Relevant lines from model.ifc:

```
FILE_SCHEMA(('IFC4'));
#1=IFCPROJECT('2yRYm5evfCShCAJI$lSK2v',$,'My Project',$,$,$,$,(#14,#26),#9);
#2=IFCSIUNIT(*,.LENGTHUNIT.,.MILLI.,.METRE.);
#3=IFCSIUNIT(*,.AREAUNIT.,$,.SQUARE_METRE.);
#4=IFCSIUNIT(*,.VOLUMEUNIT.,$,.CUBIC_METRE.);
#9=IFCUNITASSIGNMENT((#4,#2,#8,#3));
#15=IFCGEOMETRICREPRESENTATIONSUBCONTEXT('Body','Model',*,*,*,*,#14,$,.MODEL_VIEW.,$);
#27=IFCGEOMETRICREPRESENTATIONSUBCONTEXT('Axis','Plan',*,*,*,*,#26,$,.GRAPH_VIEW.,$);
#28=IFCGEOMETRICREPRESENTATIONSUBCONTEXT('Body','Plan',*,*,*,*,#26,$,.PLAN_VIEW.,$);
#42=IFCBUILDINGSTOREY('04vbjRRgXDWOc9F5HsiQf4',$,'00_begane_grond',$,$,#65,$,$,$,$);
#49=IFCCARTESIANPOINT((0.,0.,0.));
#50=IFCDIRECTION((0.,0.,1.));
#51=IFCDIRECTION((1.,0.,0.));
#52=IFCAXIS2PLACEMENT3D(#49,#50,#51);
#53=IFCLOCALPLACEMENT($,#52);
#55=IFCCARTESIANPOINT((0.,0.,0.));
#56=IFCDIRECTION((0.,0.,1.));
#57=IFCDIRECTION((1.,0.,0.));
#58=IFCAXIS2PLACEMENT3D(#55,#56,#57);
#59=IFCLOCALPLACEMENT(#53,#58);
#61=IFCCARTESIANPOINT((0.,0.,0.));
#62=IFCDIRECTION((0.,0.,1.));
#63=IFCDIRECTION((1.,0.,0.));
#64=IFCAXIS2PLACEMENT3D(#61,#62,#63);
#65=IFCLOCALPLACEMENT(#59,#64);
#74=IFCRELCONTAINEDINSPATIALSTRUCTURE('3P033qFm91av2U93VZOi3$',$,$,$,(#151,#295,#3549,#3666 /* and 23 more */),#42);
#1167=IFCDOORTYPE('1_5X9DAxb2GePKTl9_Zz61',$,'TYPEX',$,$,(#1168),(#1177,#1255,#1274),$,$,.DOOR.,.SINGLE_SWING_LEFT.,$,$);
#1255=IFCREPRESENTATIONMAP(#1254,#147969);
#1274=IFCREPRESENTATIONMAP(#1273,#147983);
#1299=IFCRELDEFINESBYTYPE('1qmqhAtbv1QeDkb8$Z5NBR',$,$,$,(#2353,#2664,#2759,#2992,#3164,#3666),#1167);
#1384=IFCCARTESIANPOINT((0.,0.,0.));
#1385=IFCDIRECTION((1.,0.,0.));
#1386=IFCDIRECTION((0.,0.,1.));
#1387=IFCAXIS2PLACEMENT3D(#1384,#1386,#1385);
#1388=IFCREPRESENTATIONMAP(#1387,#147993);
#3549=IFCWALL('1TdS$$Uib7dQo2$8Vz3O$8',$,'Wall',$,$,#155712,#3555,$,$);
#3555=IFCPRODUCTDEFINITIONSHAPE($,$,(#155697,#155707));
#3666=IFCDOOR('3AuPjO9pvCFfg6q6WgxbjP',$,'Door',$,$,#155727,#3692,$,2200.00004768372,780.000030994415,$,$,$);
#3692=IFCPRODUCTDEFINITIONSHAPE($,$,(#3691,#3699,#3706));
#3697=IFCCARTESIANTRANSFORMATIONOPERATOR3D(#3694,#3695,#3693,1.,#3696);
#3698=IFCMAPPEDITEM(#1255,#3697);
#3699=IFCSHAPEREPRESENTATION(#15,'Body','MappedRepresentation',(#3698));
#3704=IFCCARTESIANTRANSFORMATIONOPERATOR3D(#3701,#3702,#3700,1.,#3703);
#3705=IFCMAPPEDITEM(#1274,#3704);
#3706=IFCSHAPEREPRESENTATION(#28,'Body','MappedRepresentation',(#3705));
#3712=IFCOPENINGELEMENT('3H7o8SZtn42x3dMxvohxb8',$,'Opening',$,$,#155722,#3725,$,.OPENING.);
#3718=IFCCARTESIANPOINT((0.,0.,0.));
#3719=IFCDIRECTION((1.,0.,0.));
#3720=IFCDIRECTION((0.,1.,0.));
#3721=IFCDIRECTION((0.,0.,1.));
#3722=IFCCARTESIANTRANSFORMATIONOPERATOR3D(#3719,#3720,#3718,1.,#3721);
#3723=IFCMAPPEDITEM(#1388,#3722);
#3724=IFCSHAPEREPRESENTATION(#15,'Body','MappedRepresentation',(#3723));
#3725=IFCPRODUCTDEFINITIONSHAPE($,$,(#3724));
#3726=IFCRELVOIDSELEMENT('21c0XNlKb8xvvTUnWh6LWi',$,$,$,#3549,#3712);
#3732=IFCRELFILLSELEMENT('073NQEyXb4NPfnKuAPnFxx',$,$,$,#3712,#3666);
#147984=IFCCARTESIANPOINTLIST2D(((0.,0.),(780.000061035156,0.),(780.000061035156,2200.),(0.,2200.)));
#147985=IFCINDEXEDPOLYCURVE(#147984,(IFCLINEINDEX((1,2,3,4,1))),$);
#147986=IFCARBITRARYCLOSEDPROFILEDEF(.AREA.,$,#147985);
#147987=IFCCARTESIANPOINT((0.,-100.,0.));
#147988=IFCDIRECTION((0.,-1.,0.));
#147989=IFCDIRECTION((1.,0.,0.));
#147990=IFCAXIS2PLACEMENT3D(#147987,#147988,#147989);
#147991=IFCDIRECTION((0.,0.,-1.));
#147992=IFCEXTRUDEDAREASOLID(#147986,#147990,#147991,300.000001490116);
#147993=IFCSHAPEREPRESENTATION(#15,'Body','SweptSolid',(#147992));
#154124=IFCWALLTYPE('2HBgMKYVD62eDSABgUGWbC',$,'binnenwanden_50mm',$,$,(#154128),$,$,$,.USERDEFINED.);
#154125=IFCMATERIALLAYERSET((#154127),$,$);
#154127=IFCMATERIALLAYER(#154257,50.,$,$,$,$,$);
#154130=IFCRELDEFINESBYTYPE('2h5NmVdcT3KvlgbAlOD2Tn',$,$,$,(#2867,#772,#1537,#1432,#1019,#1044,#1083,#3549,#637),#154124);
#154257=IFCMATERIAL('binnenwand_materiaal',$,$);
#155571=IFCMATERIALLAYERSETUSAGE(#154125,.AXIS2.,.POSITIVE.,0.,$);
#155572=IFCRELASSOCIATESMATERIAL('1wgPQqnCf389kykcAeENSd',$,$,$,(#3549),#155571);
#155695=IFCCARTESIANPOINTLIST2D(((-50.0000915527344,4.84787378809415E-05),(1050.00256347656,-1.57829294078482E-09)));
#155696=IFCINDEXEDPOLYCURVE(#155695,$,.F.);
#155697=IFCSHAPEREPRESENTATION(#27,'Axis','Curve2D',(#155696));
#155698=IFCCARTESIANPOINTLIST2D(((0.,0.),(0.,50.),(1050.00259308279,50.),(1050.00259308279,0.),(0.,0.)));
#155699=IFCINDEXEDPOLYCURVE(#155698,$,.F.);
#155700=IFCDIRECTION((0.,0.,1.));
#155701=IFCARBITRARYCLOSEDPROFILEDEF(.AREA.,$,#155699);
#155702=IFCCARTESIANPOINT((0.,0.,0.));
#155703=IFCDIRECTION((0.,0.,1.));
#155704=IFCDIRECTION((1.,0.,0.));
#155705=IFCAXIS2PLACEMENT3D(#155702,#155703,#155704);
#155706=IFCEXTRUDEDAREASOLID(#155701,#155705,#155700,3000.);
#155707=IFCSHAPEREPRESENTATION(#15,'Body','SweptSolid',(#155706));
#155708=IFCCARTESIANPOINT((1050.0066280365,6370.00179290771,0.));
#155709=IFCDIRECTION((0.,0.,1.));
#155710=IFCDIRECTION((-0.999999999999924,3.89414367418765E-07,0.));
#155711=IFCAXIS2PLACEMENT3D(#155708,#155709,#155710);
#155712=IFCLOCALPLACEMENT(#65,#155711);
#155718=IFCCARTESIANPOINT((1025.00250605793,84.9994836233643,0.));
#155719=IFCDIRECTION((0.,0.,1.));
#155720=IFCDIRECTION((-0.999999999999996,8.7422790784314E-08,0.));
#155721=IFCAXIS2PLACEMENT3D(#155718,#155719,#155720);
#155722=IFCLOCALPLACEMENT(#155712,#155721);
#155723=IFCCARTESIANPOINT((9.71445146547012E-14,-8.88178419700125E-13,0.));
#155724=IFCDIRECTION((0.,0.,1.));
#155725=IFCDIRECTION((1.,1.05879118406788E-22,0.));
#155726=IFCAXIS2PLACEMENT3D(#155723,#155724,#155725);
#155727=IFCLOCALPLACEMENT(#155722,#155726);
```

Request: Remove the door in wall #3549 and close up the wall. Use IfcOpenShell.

```python
import ifcopenshell
import ifcopenshell.api.feature
import ifcopenshell.api.root
import ifcopenshell.geom
import ifcopenshell.util.shape

model = ifcopenshell.open("model.ifc")
settings = ifcopenshell.geom.settings()


def volume(element):
    """Net volume in cubic metres, openings subtracted."""
    shape = ifcopenshell.geom.create_shape(settings, element)
    return ifcopenshell.util.shape.get_volume(shape.geometry)


door = model.by_guid("3AuPjO9pvCFfg6q6WgxbjP")
opening = door.FillsVoids[0].RelatingOpeningElement
wall = opening.VoidsElements[0].RelatingBuildingElement
before = volume(wall)

ifcopenshell.api.root.remove_product(model, product=door)
ifcopenshell.api.feature.remove_feature(model, feature=opening)

after = volume(wall)

print(f"wall volume {before:.3f} -> {after:.3f} m3")

model.write("model_v2.ifc")
```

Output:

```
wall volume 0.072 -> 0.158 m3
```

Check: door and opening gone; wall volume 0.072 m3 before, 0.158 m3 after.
